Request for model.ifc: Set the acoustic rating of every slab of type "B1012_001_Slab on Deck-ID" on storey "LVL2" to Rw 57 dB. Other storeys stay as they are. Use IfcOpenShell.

First a look at what the model holds.

```python
import ifcopenshell
import ifcopenshell.util.element

model = ifcopenshell.open("model.ifc")
print(model.schema)
storey = next(s for s in model.by_type("IfcBuildingStorey") if s.Name == "LVL2")
slabs = [e for e in ifcopenshell.util.element.get_decomposition(storey) if e.is_a("IfcSlab")]
seen = {}
for e in slabs:
    element_type = ifcopenshell.util.element.get_type(e)
    key = (element_type.Name if element_type != e and element_type else None, ifcopenshell.util.element.get_pset(e, "Pset_SlabCommon", "AcousticRating"))
    seen[key] = seen.get(key, 0) + 1
for (name, value), count in sorted(seen.items(), key=str):
    print(count, "x", name, "|", value)
```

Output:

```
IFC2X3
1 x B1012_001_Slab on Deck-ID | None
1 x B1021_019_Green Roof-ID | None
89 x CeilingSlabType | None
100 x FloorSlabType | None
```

```python
import ifcopenshell
import ifcopenshell.api.pset
import ifcopenshell.util.element

model = ifcopenshell.open("model.ifc")

storey = next(s for s in model.by_type("IfcBuildingStorey") if s.Name == "LVL2")
slabs = [e for e in ifcopenshell.util.element.get_decomposition(storey) if e.is_a("IfcSlab")]

count = 0
for e in slabs:
    element_type = ifcopenshell.util.element.get_type(e)
    if element_type in (None, e) or element_type.Name != "B1012_001_Slab on Deck-ID":
        continue
    # add_pset returns the element's existing set when there is one.
    pset = ifcopenshell.api.pset.add_pset(model, product=e, name="Pset_SlabCommon")
    ifcopenshell.api.pset.edit_pset(model, pset=pset, properties={"AcousticRating": "Rw 57 dB"})
    count += 1

print(count, "slabs updated")

model.write("model_edited.ifc")
```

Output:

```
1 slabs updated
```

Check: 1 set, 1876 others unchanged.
